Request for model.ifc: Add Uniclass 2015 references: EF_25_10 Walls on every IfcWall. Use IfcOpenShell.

First a look at what the model holds.

```python
import ifcopenshell

model = ifcopenshell.open("model.ifc")
print(model.schema)
print("classifications:", [c.Name for c in model.by_type("IfcClassification")])
for ifc_class in ("IfcDoor", "IfcRoof", "IfcStair", "IfcWall", "IfcWindow"):
    print(ifc_class, len(model.by_type(ifc_class)))
```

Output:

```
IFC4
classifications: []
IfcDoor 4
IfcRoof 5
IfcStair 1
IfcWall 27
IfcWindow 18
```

```python
import ifcopenshell
import ifcopenshell.api.classification

model = ifcopenshell.open("model.ifc")

system = ifcopenshell.api.classification.add_classification(model, classification="Uniclass 2015")

codes = {
    "IfcWall": ("EF_25_10", "Walls"),
}
for ifc_class, (code, name) in codes.items():
    products = model.by_type(ifc_class)
    ifcopenshell.api.classification.add_reference(
        model, products=products, classification=system, identification=code, name=name
    )
    print(code, len(products))

model.write("model_edited.ifc")
```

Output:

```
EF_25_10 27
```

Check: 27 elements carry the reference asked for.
